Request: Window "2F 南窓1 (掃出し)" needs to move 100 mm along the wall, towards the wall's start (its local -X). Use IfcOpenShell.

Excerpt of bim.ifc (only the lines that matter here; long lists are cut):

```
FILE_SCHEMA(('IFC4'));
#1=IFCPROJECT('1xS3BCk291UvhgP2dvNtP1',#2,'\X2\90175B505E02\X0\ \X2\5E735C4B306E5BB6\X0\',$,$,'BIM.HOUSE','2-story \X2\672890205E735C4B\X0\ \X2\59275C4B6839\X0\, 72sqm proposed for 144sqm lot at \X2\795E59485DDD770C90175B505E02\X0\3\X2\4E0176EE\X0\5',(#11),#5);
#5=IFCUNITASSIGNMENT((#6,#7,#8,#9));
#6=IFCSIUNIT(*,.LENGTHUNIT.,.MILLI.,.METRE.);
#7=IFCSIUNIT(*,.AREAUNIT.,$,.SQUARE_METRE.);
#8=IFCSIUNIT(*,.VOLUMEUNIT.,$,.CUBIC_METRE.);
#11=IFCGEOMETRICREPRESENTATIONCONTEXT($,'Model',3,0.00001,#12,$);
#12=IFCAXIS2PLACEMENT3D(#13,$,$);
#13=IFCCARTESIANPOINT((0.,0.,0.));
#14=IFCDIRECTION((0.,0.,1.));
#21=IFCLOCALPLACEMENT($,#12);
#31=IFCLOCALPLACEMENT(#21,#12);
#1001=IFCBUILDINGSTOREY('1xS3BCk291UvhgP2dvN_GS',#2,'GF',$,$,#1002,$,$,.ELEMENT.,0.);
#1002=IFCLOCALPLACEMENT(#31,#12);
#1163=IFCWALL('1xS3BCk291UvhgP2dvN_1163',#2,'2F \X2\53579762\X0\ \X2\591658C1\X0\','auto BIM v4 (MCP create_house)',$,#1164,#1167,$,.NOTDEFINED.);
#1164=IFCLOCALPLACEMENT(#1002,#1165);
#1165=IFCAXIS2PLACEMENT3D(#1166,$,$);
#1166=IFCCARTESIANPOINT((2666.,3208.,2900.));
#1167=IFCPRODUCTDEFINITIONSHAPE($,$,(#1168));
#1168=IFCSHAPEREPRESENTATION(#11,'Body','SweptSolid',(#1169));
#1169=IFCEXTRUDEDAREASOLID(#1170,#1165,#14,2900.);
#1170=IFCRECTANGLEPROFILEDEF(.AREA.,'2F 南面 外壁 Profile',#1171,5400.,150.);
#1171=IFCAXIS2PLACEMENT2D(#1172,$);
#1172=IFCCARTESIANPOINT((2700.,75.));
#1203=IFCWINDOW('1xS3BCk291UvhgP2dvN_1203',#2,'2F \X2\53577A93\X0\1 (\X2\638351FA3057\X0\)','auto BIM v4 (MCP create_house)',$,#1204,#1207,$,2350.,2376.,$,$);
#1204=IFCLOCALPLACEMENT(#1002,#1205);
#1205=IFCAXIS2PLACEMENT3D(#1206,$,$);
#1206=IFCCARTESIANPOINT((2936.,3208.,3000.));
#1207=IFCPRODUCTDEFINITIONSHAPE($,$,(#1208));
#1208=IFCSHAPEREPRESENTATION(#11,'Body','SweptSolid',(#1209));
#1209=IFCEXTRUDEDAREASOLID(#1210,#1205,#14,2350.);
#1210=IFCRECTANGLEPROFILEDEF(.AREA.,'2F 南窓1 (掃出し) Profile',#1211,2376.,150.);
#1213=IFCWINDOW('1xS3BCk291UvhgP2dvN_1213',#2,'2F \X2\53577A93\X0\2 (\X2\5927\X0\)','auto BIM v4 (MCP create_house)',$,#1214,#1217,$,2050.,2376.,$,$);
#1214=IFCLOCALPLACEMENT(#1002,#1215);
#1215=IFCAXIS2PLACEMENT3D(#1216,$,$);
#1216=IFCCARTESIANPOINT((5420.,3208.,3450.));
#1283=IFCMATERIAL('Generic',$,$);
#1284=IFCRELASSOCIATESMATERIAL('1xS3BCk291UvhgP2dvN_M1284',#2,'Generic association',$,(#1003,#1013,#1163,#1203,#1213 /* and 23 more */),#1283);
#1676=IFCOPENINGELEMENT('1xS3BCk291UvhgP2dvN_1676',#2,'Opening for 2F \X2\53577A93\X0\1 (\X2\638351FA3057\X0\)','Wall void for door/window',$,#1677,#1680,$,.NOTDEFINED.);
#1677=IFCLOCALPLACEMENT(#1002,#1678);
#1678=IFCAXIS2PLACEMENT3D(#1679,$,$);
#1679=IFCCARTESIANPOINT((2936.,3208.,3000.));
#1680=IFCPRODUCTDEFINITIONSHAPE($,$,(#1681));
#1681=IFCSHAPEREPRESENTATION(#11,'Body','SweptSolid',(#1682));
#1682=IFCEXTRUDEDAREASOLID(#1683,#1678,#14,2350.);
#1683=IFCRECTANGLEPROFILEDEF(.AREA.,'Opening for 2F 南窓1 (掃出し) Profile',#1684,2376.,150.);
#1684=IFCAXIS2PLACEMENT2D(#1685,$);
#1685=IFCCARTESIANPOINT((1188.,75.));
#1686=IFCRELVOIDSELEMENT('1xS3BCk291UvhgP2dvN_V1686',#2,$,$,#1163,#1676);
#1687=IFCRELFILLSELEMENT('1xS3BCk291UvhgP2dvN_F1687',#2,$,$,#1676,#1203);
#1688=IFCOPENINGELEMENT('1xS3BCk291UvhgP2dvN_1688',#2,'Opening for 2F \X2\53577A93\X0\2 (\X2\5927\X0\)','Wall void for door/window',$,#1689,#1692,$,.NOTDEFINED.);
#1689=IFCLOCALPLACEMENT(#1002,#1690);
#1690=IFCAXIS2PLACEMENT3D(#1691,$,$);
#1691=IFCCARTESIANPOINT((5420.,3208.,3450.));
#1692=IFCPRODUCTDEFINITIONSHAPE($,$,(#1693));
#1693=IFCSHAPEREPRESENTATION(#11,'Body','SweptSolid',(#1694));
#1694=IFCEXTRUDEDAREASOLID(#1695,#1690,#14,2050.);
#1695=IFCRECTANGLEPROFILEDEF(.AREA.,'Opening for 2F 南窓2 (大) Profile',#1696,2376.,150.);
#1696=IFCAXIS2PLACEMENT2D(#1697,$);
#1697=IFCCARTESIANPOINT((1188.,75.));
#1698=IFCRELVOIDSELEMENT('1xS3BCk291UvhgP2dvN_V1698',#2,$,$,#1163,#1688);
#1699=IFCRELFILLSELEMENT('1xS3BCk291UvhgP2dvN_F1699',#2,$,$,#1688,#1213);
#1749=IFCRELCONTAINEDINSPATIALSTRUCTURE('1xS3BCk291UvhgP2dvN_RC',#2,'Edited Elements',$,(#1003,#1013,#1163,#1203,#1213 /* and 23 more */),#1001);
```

```python
import ifcopenshell
import ifcopenshell.api.geometry
import ifcopenshell.util.placement

model = ifcopenshell.open("bim.ifc")

window = model.by_guid("1xS3BCk291UvhgP2dvN_1203")
opening = window.FillsVoids[0].RelatingOpeningElement
wall = opening.VoidsElements[0].RelatingBuildingElement

wall_matrix = ifcopenshell.util.placement.get_local_placement(wall.ObjectPlacement)
shift = wall_matrix[:3, 0] * -100.0
before = ifcopenshell.util.placement.get_local_placement(window.ObjectPlacement)[:3, 3].copy()

# The window is not placed relative to its opening, so move both.
for product in (opening, window):
    matrix = ifcopenshell.util.placement.get_local_placement(product.ObjectPlacement)
    matrix[:3, 3] += shift
    ifcopenshell.api.geometry.edit_object_placement(model, product=product, matrix=matrix, is_si=False)

after = ifcopenshell.util.placement.get_local_placement(window.ObjectPlacement)[:3, 3]
print("window moved by", (after - before).round(3) + 0.0)

model.write("bim_rev.ifc")
```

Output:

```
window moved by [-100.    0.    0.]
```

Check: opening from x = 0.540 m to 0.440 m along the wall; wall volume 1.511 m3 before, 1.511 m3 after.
